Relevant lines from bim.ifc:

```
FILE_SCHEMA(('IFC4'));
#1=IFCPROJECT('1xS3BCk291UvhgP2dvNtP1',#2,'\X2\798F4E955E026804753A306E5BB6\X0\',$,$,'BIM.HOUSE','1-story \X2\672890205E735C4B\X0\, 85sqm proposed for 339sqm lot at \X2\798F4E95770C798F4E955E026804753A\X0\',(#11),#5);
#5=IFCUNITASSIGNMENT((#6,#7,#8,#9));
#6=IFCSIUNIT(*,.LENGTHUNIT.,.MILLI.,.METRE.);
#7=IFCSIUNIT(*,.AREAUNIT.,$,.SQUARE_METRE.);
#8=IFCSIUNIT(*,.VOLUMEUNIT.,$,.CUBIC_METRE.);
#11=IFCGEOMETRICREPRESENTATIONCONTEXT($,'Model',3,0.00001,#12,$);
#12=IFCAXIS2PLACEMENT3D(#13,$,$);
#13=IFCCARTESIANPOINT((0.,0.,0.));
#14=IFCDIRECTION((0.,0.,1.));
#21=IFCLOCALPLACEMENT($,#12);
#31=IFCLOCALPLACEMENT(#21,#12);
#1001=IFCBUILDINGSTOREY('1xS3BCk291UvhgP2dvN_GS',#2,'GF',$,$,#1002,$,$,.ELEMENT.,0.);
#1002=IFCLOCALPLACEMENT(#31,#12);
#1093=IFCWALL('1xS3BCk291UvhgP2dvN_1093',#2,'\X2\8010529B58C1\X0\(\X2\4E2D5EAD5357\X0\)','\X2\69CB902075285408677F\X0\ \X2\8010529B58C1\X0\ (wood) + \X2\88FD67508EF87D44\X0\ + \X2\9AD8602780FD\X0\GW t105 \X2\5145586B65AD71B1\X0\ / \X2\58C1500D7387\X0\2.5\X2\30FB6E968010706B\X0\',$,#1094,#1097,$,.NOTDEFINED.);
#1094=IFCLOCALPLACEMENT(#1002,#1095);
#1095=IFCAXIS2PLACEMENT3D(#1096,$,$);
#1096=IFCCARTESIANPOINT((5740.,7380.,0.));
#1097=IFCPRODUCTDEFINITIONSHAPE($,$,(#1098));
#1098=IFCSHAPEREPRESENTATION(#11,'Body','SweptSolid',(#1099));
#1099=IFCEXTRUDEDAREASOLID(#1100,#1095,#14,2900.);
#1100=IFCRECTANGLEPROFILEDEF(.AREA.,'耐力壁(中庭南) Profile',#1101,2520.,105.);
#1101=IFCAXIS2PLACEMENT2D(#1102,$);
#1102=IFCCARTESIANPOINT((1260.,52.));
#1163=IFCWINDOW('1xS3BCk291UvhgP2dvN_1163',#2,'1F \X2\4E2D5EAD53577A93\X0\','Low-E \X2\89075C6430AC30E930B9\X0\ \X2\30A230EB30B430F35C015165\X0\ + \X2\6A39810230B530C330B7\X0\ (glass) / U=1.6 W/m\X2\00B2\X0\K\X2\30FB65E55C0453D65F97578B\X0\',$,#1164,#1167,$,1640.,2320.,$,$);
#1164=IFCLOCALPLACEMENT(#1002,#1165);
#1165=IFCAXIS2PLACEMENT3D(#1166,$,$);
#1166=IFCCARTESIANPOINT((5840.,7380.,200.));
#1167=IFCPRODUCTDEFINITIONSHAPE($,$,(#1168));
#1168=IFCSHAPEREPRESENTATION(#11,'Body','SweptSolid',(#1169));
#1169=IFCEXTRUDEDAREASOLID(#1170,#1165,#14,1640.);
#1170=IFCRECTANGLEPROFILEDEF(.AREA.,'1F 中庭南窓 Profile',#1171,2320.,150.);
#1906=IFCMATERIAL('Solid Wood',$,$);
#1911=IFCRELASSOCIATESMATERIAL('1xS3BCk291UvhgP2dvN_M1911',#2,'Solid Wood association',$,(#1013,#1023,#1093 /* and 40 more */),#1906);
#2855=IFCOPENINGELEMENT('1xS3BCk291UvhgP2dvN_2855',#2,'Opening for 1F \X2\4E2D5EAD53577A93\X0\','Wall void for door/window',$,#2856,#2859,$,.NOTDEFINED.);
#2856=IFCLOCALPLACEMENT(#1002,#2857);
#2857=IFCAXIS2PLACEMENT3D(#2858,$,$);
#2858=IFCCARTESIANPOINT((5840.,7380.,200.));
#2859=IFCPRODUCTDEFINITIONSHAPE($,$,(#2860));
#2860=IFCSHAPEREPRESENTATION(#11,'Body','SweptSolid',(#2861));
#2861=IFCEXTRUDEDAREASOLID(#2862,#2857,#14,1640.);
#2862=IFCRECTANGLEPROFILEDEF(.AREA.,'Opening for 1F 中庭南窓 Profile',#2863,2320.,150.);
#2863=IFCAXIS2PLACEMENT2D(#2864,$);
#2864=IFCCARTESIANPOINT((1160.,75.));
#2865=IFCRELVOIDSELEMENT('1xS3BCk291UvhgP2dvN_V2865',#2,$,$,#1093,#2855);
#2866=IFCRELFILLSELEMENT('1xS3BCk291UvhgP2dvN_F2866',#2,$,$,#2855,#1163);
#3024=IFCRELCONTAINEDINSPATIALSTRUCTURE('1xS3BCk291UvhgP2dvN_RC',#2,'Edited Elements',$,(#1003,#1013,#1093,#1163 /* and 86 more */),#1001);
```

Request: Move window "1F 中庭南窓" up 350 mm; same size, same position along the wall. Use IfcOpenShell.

```python
import numpy as np
import ifcopenshell
import ifcopenshell.api.geometry
import ifcopenshell.util.placement
import ifcopenshell.util.unit

model = ifcopenshell.open("bim.ifc")
unit_scale = ifcopenshell.util.unit.calculate_unit_scale(model)

window = model.by_guid("1xS3BCk291UvhgP2dvN_1163")
opening = window.FillsVoids[0].RelatingOpeningElement
dz = 0.35 / unit_scale

shift = np.array([0.0, 0.0, dz])
# The window is not placed relative to its opening, so move both.
for product in (opening, window):
    matrix = ifcopenshell.util.placement.get_local_placement(product.ObjectPlacement)
    matrix[:3, 3] += shift
    ifcopenshell.api.geometry.edit_object_placement(model, product=product, matrix=matrix, is_si=False)

print(f"moved by {dz * unit_scale:+.3f} m")

model.write("bim-out.ifc")
```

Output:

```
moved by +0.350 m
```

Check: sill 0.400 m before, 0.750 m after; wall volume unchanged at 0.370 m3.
